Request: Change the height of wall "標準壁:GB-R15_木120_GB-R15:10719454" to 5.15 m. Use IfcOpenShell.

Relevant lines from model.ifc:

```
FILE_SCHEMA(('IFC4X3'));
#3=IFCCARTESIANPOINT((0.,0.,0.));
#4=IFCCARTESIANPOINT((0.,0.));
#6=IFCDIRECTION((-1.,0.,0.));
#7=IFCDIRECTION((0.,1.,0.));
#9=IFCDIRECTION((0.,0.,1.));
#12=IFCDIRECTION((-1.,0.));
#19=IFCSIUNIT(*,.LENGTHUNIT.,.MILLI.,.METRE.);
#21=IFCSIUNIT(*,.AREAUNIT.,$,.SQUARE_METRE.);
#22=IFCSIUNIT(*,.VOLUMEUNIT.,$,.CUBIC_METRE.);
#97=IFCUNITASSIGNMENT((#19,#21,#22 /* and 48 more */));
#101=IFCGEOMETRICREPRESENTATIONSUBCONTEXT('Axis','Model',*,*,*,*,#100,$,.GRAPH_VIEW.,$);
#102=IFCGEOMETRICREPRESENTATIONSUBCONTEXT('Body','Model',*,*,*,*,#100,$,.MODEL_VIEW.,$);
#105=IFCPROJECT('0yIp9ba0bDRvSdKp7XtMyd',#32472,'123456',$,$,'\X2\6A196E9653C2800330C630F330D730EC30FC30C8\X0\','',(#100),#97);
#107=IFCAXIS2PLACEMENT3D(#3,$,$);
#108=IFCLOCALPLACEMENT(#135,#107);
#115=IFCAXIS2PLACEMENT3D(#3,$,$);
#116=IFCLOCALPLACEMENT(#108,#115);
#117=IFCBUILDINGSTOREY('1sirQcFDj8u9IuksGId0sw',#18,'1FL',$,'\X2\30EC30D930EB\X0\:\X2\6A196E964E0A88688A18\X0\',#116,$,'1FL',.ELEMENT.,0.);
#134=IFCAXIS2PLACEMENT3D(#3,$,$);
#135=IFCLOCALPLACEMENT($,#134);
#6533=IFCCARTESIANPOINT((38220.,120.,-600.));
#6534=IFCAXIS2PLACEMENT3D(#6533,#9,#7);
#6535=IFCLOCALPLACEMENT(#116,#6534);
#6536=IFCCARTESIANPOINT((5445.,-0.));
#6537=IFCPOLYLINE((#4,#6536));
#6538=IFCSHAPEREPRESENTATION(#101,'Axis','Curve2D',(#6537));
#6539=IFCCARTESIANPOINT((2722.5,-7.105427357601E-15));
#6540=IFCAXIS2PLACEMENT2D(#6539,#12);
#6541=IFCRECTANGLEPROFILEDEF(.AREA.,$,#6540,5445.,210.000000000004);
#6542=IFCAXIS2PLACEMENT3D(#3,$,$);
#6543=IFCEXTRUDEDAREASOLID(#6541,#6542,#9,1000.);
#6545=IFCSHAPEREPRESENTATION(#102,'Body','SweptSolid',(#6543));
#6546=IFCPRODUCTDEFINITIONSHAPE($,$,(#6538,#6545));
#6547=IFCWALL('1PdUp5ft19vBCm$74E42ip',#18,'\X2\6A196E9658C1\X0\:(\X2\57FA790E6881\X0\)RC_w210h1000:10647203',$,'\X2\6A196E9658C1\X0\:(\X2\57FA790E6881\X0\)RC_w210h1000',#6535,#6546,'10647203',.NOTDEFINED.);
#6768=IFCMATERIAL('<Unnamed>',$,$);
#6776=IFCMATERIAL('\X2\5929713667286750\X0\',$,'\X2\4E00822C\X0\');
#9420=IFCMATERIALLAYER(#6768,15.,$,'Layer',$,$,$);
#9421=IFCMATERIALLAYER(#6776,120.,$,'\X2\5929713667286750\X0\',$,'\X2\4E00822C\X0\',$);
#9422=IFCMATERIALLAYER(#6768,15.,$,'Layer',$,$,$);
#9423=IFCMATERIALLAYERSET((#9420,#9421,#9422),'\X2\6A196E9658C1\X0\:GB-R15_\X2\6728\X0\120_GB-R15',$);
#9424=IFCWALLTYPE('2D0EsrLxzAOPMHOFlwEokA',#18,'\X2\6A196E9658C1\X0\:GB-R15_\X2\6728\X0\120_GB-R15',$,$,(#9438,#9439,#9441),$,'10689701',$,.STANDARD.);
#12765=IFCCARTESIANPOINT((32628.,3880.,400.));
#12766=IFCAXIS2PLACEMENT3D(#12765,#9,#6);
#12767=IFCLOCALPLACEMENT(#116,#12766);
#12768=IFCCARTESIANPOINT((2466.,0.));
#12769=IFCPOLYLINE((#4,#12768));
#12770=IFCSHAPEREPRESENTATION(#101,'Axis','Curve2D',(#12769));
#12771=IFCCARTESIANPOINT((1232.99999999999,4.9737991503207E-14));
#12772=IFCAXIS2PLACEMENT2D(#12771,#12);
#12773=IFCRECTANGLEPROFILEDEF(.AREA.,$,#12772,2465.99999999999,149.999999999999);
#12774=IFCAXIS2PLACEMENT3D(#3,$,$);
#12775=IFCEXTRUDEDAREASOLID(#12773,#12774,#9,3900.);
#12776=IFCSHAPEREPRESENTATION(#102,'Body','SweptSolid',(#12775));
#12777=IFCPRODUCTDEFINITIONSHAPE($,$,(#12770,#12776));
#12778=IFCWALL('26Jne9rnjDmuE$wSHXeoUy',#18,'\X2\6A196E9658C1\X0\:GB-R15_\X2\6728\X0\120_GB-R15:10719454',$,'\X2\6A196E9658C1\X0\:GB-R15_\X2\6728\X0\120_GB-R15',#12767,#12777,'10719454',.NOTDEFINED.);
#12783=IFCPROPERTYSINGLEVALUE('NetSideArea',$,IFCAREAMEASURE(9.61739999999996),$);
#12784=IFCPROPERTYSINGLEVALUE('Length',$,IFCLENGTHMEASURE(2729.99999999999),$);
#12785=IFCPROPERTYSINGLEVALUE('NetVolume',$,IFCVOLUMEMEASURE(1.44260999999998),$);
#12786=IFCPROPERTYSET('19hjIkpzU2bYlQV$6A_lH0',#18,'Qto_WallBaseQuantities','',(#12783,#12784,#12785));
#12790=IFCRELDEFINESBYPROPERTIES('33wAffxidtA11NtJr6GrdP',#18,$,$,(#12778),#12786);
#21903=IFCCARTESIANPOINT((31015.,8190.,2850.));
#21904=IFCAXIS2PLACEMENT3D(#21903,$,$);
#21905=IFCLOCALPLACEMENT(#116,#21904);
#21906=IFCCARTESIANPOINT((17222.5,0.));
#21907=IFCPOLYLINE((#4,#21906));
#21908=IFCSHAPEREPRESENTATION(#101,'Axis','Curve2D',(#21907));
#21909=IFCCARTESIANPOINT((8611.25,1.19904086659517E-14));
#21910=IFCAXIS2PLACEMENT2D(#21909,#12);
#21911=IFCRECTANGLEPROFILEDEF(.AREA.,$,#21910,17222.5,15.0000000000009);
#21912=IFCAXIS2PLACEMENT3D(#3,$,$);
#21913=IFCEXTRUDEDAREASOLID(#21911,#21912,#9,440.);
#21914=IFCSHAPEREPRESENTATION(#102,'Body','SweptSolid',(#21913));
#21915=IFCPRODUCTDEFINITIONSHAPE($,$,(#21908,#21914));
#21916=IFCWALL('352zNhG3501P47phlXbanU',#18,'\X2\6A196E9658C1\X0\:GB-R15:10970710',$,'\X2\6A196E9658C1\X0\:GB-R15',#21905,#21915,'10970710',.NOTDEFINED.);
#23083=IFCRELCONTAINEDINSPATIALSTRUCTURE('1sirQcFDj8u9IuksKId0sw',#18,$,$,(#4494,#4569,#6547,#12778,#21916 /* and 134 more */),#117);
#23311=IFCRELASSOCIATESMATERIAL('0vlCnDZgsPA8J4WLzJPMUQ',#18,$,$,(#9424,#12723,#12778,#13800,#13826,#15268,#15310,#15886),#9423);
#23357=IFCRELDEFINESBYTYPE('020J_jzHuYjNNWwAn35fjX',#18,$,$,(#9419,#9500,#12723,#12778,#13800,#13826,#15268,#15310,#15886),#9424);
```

```python
import ifcopenshell
import ifcopenshell.api.pset
import ifcopenshell.geom
import ifcopenshell.util.element
import ifcopenshell.util.representation
import ifcopenshell.util.shape
import ifcopenshell.util.unit

model = ifcopenshell.open("model.ifc")
unit_scale = ifcopenshell.util.unit.calculate_unit_scale(model)
area_scale = ifcopenshell.util.unit.calculate_unit_scale(model, "AREAUNIT")
volume_scale = ifcopenshell.util.unit.calculate_unit_scale(model, "VOLUMEUNIT")
settings = ifcopenshell.geom.settings()


def volume(element):
    """Net volume in cubic metres, openings subtracted."""
    shape = ifcopenshell.geom.create_shape(settings, element)
    return ifcopenshell.util.shape.get_volume(shape.geometry)


wall = model.by_guid("26Jne9rnjDmuE$wSHXeoUy")
before = volume(wall)

body = ifcopenshell.util.representation.get_representation(wall, "Model", "Body")
solid = body.Items[0]
old_height = solid.Depth
solid.Depth = 5.15 / unit_scale
after = volume(wall)
thickness = 0.15  # wall thickness in metres

# Update the stored height, areas and volumes.
pset = model.by_id(ifcopenshell.util.element.get_pset(wall, "Qto_WallBaseQuantities", should_inherit=False)["id"])
ifcopenshell.api.pset.edit_pset(model, pset=pset, properties={
    "NetSideArea": model.create_entity("IfcAreaMeasure", after / thickness / area_scale),
    "NetVolume": model.create_entity("IfcVolumeMeasure", after / volume_scale),
})

print(f"height {old_height:g} -> {solid.Depth:g}, volume {before:.3f} -> {after:.3f} m3")

model.write("model_rev.ifc")
```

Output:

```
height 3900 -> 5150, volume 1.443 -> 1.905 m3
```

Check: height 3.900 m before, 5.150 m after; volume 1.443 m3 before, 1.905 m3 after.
